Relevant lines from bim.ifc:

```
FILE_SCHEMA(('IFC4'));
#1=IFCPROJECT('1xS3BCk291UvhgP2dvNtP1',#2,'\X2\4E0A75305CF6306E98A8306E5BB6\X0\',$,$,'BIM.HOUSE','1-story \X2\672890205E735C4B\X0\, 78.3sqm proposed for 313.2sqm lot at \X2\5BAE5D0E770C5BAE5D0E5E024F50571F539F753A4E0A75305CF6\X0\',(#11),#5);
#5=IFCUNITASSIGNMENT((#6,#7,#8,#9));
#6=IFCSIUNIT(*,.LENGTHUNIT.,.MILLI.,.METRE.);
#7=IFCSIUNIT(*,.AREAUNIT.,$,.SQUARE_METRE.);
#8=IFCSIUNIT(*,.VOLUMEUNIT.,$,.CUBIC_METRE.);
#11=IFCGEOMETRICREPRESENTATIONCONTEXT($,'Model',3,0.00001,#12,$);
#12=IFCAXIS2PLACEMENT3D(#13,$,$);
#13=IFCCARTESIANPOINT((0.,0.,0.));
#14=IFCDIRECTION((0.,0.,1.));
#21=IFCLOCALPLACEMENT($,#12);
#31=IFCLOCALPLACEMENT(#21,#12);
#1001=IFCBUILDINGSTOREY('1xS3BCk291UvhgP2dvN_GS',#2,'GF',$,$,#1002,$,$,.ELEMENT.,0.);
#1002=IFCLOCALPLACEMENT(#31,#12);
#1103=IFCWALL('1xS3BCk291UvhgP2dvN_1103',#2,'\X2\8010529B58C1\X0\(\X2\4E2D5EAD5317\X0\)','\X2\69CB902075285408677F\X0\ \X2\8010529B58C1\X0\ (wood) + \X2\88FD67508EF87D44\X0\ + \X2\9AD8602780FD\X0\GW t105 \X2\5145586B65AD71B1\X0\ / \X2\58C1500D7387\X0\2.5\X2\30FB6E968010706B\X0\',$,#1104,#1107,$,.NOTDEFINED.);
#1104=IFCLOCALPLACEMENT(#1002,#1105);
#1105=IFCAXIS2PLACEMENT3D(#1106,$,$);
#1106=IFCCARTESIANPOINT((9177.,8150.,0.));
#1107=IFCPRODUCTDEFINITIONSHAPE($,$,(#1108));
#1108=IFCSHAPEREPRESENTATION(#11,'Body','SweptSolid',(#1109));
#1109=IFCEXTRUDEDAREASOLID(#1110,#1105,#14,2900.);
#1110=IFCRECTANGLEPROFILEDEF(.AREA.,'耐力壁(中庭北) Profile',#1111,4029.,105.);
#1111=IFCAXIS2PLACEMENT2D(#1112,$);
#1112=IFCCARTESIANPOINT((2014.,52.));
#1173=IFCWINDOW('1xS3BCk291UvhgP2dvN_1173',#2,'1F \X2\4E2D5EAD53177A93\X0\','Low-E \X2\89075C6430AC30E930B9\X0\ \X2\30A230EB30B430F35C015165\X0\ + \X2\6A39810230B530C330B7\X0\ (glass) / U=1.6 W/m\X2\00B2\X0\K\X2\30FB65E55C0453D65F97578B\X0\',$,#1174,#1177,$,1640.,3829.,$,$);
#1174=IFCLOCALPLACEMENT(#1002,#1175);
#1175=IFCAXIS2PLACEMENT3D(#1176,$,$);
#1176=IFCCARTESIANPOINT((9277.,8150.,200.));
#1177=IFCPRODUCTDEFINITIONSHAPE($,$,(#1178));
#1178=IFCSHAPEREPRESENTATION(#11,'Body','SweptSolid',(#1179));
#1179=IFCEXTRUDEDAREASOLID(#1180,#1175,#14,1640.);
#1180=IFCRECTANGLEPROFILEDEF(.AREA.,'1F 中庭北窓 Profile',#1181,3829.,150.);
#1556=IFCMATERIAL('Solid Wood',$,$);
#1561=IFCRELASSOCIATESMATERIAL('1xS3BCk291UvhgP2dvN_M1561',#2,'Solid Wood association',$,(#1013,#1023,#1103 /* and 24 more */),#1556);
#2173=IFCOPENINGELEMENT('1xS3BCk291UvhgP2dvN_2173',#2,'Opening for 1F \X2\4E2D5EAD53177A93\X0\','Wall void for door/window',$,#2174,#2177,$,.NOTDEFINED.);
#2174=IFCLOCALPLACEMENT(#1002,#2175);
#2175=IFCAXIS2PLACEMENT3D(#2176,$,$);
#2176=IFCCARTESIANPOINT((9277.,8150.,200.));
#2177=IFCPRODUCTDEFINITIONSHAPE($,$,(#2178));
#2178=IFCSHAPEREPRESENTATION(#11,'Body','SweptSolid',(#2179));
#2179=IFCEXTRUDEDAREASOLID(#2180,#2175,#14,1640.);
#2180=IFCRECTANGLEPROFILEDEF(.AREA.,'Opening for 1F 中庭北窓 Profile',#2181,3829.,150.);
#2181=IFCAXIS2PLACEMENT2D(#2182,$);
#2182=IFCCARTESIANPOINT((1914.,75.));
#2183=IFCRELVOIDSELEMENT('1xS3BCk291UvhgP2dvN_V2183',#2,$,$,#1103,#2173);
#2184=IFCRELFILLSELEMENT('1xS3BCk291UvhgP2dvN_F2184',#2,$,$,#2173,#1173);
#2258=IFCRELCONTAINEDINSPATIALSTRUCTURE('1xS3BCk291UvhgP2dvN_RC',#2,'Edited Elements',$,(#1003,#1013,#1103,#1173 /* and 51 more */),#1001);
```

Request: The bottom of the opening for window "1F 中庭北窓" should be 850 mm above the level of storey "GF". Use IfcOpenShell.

```python
import numpy as np
import ifcopenshell
import ifcopenshell.api.geometry
import ifcopenshell.geom
import ifcopenshell.util.element
import ifcopenshell.util.placement
import ifcopenshell.util.shape
import ifcopenshell.util.unit

model = ifcopenshell.open("bim.ifc")
unit_scale = ifcopenshell.util.unit.calculate_unit_scale(model)

window = model.by_guid("1xS3BCk291UvhgP2dvN_1173")
opening = window.FillsVoids[0].RelatingOpeningElement
storey = ifcopenshell.util.element.get_container(window, ifc_class="IfcBuildingStorey")
level = ifcopenshell.util.placement.get_local_placement(storey.ObjectPlacement)[2, 3]

# The opening's origin need not be at the sill, so measure its lowest point.
shape = ifcopenshell.geom.create_shape(ifcopenshell.geom.settings(), opening)
bottom = ifcopenshell.util.shape.get_shape_bottom_elevation(shape, shape.geometry) / unit_scale
dz = level + 0.85 / unit_scale - bottom

shift = np.array([0.0, 0.0, dz])
# The window is not placed relative to its opening, so move both.
for product in (opening, window):
    matrix = ifcopenshell.util.placement.get_local_placement(product.ObjectPlacement)
    matrix[:3, 3] += shift
    ifcopenshell.api.geometry.edit_object_placement(model, product=product, matrix=matrix, is_si=False)

print(f"moved by {dz * unit_scale:+.3f} m")

model.write("bim-out.ifc")
```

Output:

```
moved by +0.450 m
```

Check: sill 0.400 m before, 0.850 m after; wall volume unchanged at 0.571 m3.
